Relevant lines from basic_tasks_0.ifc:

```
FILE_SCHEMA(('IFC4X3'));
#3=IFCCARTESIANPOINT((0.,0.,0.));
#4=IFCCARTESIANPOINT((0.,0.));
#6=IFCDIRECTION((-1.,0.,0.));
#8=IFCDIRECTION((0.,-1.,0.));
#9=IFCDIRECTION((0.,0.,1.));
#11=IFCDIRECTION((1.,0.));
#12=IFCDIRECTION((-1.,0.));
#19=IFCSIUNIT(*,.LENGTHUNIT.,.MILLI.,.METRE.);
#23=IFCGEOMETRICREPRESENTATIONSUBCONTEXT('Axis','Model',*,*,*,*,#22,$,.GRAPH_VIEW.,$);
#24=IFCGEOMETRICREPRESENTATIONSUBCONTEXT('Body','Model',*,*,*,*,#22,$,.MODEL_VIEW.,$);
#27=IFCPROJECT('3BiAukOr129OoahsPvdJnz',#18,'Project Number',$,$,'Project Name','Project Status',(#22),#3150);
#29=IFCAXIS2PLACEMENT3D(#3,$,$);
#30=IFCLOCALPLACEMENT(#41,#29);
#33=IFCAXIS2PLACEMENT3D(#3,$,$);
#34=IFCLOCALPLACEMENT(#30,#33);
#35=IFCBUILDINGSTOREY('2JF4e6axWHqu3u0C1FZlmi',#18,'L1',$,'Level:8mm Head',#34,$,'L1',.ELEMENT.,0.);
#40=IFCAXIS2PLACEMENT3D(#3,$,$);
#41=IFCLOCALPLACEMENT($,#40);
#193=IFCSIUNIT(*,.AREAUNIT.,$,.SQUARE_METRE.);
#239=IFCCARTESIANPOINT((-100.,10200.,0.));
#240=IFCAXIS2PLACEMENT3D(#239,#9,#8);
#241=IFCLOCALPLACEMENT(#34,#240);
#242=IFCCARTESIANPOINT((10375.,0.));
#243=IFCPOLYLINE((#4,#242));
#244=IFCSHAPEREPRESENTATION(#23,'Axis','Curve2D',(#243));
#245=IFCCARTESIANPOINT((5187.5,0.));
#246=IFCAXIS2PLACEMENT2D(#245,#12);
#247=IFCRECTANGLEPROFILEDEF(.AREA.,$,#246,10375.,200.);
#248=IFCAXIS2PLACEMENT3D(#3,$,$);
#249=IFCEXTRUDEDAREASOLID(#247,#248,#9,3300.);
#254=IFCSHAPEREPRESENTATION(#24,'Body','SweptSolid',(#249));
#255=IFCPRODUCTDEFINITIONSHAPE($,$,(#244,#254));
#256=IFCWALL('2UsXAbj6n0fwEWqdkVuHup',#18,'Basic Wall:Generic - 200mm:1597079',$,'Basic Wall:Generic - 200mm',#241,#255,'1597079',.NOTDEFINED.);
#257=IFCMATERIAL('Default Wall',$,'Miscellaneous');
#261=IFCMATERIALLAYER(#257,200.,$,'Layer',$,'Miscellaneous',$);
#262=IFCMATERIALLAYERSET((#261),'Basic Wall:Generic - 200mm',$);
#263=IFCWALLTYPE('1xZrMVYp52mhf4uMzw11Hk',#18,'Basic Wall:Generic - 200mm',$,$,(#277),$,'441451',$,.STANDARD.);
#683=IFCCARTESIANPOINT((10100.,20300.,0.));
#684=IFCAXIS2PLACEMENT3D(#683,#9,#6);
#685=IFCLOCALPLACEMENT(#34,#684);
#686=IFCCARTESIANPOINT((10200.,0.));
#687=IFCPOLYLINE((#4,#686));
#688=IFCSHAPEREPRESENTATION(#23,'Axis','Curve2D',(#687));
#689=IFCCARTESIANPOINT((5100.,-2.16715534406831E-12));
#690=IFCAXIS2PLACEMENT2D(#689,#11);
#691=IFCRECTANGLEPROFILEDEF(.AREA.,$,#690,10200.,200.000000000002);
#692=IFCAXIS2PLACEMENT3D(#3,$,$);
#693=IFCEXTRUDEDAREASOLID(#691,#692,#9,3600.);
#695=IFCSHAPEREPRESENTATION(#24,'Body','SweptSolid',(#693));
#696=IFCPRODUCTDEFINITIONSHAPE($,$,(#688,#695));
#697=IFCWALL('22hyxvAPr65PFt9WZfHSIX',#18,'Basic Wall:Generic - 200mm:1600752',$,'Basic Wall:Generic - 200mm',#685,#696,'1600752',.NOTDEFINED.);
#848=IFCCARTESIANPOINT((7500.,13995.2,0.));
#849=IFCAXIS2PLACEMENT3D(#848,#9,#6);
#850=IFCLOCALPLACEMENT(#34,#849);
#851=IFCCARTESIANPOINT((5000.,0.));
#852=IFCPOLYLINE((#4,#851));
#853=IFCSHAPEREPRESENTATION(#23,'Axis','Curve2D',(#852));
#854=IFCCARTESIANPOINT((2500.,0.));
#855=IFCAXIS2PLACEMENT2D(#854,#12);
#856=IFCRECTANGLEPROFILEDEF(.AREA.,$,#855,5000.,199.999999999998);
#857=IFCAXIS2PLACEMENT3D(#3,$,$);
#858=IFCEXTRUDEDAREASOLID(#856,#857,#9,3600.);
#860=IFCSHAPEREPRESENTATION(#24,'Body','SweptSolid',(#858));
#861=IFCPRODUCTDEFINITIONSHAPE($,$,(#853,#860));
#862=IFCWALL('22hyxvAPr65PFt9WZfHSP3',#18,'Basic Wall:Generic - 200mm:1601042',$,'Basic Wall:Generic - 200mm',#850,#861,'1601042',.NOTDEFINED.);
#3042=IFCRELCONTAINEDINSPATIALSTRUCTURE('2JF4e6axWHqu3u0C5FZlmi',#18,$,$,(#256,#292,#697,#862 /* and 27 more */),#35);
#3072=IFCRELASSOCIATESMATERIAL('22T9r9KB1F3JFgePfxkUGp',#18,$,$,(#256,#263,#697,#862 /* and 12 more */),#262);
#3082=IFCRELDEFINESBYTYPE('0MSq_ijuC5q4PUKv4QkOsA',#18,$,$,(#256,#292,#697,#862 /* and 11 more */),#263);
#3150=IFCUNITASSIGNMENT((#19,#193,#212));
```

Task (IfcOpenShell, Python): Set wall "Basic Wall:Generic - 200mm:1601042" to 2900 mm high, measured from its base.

```python
import ifcopenshell
import ifcopenshell.geom
import ifcopenshell.util.representation
import ifcopenshell.util.shape
import ifcopenshell.util.unit

model = ifcopenshell.open("basic_tasks_0.ifc")
unit_scale = ifcopenshell.util.unit.calculate_unit_scale(model)
settings = ifcopenshell.geom.settings()


def volume(element):
    """Net volume in cubic metres, openings subtracted."""
    shape = ifcopenshell.geom.create_shape(settings, element)
    return ifcopenshell.util.shape.get_volume(shape.geometry)


wall = model.by_id(862)
before = volume(wall)

body = ifcopenshell.util.representation.get_representation(wall, "Model", "Body")
solid = body.Items[0]
old_height = solid.Depth
solid.Depth = 2.9 / unit_scale
after = volume(wall)

print(f"height {old_height:g} -> {solid.Depth:g}, volume {before:.3f} -> {after:.3f} m3")

model.write("basic_tasks_0_edited.ifc")
```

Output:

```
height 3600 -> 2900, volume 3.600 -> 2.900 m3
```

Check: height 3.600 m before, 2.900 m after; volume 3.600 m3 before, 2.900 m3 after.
